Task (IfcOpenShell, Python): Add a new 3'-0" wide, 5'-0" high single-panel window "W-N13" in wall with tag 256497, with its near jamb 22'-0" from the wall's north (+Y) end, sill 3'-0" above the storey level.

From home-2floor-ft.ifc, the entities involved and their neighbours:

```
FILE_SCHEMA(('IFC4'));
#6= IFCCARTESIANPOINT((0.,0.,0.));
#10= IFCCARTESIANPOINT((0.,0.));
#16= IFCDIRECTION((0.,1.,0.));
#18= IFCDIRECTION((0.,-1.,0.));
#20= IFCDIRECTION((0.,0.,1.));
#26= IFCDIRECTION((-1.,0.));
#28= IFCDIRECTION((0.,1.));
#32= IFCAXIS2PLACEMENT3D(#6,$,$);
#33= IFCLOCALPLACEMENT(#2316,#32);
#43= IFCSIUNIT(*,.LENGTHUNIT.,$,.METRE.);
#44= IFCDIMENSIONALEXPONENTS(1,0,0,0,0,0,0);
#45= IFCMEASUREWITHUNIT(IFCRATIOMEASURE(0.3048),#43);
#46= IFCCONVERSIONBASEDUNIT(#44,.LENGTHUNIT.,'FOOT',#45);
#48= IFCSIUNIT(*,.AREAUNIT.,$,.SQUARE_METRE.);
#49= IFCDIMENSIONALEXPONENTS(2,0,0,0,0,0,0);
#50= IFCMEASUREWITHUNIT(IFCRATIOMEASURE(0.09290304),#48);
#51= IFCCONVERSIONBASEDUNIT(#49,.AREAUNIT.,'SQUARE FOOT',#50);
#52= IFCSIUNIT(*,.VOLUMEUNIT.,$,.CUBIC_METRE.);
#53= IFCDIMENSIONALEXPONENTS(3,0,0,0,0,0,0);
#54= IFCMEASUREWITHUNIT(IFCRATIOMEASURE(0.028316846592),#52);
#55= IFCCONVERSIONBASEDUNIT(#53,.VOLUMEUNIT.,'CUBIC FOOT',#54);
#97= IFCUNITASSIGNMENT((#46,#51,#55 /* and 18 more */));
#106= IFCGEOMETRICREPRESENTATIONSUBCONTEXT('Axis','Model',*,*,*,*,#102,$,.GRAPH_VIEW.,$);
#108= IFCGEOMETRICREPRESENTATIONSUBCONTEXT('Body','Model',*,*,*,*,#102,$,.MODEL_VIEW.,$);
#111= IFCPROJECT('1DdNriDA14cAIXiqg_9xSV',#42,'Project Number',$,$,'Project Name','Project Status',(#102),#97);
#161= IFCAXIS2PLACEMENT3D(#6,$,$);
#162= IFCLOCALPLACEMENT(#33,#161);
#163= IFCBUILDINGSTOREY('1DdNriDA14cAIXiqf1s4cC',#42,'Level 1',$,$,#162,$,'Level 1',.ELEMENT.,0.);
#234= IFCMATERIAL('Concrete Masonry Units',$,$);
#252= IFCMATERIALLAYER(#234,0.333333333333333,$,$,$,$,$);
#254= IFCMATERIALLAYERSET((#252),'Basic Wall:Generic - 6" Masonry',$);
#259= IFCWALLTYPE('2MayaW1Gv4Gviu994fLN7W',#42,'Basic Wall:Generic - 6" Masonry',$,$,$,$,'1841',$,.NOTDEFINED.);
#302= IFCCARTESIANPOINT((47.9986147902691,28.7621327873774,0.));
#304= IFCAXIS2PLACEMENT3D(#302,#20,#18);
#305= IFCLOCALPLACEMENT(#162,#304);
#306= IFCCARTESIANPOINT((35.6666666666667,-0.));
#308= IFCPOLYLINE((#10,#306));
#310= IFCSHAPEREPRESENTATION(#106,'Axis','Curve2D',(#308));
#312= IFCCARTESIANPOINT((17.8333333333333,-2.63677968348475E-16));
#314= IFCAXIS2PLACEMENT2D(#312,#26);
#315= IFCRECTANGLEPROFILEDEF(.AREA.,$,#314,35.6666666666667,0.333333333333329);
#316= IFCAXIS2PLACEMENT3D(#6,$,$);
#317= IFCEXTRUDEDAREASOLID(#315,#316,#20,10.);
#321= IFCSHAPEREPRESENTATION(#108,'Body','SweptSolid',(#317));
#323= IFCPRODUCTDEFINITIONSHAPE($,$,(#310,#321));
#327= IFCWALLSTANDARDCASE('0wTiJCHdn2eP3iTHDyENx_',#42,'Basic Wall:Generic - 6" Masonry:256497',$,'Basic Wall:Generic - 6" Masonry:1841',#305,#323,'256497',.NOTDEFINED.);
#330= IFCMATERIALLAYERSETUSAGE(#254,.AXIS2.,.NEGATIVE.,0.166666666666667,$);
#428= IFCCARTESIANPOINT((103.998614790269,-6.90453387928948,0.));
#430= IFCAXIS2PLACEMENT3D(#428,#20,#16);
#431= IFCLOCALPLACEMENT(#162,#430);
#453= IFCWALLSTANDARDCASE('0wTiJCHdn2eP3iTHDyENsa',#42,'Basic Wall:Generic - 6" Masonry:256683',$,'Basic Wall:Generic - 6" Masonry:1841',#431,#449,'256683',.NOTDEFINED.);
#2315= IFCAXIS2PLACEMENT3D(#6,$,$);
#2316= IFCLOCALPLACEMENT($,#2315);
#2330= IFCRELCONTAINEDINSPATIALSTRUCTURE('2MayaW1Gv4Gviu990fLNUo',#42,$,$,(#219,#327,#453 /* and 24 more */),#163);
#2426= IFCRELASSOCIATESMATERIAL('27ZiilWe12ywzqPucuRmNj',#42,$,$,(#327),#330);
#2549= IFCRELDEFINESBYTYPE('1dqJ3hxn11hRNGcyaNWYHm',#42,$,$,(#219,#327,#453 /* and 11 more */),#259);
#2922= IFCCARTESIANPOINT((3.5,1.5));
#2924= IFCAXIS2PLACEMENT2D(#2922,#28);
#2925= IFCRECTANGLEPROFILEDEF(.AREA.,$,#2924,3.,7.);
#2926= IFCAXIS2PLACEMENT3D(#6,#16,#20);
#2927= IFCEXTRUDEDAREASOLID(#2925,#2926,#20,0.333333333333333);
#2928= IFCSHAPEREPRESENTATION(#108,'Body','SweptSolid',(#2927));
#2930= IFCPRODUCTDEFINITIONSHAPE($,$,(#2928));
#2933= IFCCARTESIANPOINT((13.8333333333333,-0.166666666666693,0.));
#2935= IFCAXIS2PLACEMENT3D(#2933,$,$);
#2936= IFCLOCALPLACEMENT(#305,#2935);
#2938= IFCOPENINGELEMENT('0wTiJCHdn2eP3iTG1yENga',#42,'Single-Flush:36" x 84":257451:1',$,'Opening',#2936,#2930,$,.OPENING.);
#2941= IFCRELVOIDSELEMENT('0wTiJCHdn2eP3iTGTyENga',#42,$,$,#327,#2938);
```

```python
import numpy as np
import ifcopenshell
import ifcopenshell.api.feature
import ifcopenshell.api.geometry
import ifcopenshell.api.root
import ifcopenshell.api.spatial
import ifcopenshell.geom
import ifcopenshell.util.element
import ifcopenshell.util.placement
import ifcopenshell.util.representation
import ifcopenshell.util.shape
import ifcopenshell.util.unit

model = ifcopenshell.open("home-2floor-ft.ifc")
unit_scale = ifcopenshell.util.unit.calculate_unit_scale(model)
settings = ifcopenshell.geom.settings()


def volume(element):
    """Net volume in cubic metres, openings subtracted."""
    shape = ifcopenshell.geom.create_shape(settings, element)
    return ifcopenshell.util.shape.get_volume(shape.geometry)


wall = model.by_guid("0wTiJCHdn2eP3iTHDyENx_")
storey = ifcopenshell.util.element.get_container(wall, ifc_class="IfcBuildingStorey")
context = ifcopenshell.util.representation.get_context(model, "Model", "Body", "MODEL_VIEW")
before = volume(wall)

width, height, from_end, sill = 0.9144, 1.524, 6.7056, 0.9144  # metres

# The wall runs along its own X axis, and the end named is its -X end.
wall_shape = ifcopenshell.geom.create_shape(settings, wall)
x, y, z = ifcopenshell.util.shape.get_vertices(wall_shape.geometry).T
start = x.min() + from_end
face, thickness = float(y.min()), float(y.max() - y.min())
wall_matrix = ifcopenshell.util.placement.get_local_placement(wall.ObjectPlacement)
level = ifcopenshell.util.placement.get_local_placement(storey.ObjectPlacement)[2, 3]


def in_wall(x, y):
    """Placement at x, y metres in the wall's axes, at sill height."""
    matrix = wall_matrix.copy()
    matrix[:, 3] = wall_matrix @ np.array([x / unit_scale, y / unit_scale, 0.0, 1.0])
    matrix[2, 3] = level + sill / unit_scale
    return matrix


# Opening: a box that overshoots both wall faces by 50 mm.
opening = ifcopenshell.api.root.create_entity(model, ifc_class="IfcOpeningElement", predefined_type="OPENING")
box = ifcopenshell.api.geometry.add_wall_representation(
    model, context=context, length=width, height=height, thickness=thickness + 0.1
)
ifcopenshell.api.geometry.assign_representation(model, product=opening, representation=box)
ifcopenshell.api.geometry.edit_object_placement(model, product=opening, matrix=in_wall(start, face - 0.05), is_si=False)
ifcopenshell.api.feature.add_feature(model, feature=opening, element=wall)

window = ifcopenshell.api.root.create_entity(model, ifc_class="IfcWindow", name="W-N13", predefined_type="WINDOW")
window.OverallWidth, window.OverallHeight = width / unit_scale, height / unit_scale
window.PartitioningType = "SINGLE_PANEL"
body = ifcopenshell.api.geometry.add_window_representation(
    model,
    context=context,
    overall_width=window.OverallWidth,
    overall_height=window.OverallHeight,
    partition_type="SINGLE_PANEL",
)
ifcopenshell.api.geometry.assign_representation(model, product=window, representation=body)
ifcopenshell.api.spatial.assign_container(model, products=[window], relating_structure=storey)
ifcopenshell.api.feature.add_filling(model, opening=opening, element=window)

# Centre the window in the wall's thickness.
ifcopenshell.api.geometry.edit_object_placement(model, product=window, matrix=in_wall(start, face), is_si=False)
window_shape = ifcopenshell.geom.create_shape(settings, window)
depth = ifcopenshell.util.shape.get_vertices(window_shape.geometry)[:, 1]
offset = face + thickness / 2 - (depth.min() + depth.max()) / 2
ifcopenshell.api.geometry.edit_object_placement(model, product=window, matrix=in_wall(start, offset), is_si=False)

after = volume(wall)

print(f"wall volume {before:.3f} -> {after:.3f} m3")

model.write("home-2floor-ft_rev.ifc")
```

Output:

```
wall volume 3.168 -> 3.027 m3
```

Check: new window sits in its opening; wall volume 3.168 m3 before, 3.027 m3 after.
